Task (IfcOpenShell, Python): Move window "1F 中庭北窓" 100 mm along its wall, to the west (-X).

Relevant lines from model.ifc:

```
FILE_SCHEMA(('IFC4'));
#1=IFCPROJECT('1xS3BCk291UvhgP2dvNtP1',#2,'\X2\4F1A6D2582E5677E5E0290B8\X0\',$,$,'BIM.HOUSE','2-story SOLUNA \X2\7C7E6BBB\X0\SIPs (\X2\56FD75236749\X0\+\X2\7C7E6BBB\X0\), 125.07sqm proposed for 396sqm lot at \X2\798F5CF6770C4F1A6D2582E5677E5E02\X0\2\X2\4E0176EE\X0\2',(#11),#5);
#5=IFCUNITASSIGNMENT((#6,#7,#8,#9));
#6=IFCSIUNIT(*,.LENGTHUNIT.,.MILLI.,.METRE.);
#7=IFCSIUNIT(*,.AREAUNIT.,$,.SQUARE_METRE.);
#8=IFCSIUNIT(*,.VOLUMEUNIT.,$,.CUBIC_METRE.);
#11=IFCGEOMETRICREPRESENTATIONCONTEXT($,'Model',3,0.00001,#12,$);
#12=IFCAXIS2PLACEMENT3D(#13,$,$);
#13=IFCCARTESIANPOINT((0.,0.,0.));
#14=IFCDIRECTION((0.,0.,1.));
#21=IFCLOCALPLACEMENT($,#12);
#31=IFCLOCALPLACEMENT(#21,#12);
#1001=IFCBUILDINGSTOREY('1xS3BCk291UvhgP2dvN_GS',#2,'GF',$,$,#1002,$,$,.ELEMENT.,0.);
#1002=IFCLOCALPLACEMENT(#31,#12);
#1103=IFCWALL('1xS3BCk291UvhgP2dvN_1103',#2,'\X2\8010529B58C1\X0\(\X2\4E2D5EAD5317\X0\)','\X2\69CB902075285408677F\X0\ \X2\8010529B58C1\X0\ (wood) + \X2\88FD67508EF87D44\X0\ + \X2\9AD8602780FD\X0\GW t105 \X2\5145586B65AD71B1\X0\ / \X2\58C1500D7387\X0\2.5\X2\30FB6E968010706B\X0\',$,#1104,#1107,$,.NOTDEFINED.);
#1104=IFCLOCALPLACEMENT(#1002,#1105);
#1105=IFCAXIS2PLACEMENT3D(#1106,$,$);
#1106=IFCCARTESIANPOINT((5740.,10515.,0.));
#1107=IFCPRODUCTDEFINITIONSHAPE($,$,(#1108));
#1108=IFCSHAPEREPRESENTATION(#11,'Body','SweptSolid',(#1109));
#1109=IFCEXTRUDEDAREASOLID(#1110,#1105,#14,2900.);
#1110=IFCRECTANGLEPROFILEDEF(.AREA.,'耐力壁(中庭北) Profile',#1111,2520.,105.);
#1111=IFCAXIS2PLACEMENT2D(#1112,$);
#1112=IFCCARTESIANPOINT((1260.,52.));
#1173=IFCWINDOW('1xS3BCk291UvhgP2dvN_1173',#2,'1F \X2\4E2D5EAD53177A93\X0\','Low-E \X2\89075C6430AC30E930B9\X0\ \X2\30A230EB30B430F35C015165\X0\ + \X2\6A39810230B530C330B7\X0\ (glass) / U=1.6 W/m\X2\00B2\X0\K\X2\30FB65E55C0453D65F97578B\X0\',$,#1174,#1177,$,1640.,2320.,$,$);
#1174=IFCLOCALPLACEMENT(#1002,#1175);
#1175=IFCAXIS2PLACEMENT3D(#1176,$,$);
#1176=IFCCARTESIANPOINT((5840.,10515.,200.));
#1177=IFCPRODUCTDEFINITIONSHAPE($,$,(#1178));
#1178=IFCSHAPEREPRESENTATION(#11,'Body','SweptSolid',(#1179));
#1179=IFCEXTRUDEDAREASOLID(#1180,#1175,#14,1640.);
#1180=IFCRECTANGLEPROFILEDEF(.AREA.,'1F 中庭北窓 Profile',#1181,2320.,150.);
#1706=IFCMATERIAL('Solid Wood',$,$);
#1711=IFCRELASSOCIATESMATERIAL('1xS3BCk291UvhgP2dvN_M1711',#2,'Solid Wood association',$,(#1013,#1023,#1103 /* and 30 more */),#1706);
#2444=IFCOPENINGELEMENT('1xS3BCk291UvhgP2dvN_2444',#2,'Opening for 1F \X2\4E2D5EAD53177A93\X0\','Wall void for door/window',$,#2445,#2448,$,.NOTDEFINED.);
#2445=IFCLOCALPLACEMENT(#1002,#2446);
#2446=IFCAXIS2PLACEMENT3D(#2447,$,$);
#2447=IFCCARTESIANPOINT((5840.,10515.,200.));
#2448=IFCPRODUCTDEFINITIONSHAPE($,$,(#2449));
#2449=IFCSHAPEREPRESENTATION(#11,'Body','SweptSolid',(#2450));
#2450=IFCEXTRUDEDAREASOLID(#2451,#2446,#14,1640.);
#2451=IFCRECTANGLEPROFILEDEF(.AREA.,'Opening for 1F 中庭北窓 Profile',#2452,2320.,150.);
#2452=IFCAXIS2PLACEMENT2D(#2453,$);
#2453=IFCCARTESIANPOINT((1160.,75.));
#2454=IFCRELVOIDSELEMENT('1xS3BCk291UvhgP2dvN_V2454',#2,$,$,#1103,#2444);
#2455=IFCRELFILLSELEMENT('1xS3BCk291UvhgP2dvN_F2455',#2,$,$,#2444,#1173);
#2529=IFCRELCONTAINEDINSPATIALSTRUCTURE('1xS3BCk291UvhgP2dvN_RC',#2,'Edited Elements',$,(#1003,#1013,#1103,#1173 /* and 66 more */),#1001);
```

```python
import ifcopenshell
import ifcopenshell.api.geometry
import ifcopenshell.util.placement

model = ifcopenshell.open("model.ifc")

window = model.by_guid("1xS3BCk291UvhgP2dvN_1173")
opening = window.FillsVoids[0].RelatingOpeningElement
wall = opening.VoidsElements[0].RelatingBuildingElement

wall_matrix = ifcopenshell.util.placement.get_local_placement(wall.ObjectPlacement)
shift = wall_matrix[:3, 0] * -100.0
before = ifcopenshell.util.placement.get_local_placement(window.ObjectPlacement)[:3, 3].copy()

# The window is not placed relative to its opening, so move both.
for product in (opening, window):
    matrix = ifcopenshell.util.placement.get_local_placement(product.ObjectPlacement)
    matrix[:3, 3] += shift
    ifcopenshell.api.geometry.edit_object_placement(model, product=product, matrix=matrix, is_si=False)

after = ifcopenshell.util.placement.get_local_placement(window.ObjectPlacement)[:3, 3]
print("window moved by", (after - before).round(3) + 0.0)

model.write("model_rev.ifc")
```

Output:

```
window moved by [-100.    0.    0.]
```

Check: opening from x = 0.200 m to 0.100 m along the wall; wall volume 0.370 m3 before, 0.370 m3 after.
